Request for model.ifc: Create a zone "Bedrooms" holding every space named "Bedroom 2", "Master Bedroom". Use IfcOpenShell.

First a look at what the model holds.

```python
import ifcopenshell

model = ifcopenshell.open("model.ifc")
print(model.schema)
seen = {}
for space in model.by_type("IfcSpace"):
    seen[space.LongName] = seen.get(space.LongName, 0) + 1
for name, count in sorted(seen.items(), key=str):
    print(count, "x", name)
print("zones:", [z.Name for z in model.by_type("IfcZone")][:20])
```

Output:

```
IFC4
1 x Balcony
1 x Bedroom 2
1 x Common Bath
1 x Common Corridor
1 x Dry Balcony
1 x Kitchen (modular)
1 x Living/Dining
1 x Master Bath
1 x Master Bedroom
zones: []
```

```python
import ifcopenshell
import ifcopenshell.api.group
import ifcopenshell.api.root

model = ifcopenshell.open("model.ifc")

names = {"Bedroom 2", "Master Bedroom"}
spaces = [s for s in model.by_type("IfcSpace") if s.LongName in names]

zone = ifcopenshell.api.root.create_entity(model, ifc_class="IfcZone", name="Bedrooms")
ifcopenshell.api.group.assign_group(model, products=spaces, group=zone)
print(len(spaces), "spaces in", zone.Name)

model.write("model_updated.ifc")
```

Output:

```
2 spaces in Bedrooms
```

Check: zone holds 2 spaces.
